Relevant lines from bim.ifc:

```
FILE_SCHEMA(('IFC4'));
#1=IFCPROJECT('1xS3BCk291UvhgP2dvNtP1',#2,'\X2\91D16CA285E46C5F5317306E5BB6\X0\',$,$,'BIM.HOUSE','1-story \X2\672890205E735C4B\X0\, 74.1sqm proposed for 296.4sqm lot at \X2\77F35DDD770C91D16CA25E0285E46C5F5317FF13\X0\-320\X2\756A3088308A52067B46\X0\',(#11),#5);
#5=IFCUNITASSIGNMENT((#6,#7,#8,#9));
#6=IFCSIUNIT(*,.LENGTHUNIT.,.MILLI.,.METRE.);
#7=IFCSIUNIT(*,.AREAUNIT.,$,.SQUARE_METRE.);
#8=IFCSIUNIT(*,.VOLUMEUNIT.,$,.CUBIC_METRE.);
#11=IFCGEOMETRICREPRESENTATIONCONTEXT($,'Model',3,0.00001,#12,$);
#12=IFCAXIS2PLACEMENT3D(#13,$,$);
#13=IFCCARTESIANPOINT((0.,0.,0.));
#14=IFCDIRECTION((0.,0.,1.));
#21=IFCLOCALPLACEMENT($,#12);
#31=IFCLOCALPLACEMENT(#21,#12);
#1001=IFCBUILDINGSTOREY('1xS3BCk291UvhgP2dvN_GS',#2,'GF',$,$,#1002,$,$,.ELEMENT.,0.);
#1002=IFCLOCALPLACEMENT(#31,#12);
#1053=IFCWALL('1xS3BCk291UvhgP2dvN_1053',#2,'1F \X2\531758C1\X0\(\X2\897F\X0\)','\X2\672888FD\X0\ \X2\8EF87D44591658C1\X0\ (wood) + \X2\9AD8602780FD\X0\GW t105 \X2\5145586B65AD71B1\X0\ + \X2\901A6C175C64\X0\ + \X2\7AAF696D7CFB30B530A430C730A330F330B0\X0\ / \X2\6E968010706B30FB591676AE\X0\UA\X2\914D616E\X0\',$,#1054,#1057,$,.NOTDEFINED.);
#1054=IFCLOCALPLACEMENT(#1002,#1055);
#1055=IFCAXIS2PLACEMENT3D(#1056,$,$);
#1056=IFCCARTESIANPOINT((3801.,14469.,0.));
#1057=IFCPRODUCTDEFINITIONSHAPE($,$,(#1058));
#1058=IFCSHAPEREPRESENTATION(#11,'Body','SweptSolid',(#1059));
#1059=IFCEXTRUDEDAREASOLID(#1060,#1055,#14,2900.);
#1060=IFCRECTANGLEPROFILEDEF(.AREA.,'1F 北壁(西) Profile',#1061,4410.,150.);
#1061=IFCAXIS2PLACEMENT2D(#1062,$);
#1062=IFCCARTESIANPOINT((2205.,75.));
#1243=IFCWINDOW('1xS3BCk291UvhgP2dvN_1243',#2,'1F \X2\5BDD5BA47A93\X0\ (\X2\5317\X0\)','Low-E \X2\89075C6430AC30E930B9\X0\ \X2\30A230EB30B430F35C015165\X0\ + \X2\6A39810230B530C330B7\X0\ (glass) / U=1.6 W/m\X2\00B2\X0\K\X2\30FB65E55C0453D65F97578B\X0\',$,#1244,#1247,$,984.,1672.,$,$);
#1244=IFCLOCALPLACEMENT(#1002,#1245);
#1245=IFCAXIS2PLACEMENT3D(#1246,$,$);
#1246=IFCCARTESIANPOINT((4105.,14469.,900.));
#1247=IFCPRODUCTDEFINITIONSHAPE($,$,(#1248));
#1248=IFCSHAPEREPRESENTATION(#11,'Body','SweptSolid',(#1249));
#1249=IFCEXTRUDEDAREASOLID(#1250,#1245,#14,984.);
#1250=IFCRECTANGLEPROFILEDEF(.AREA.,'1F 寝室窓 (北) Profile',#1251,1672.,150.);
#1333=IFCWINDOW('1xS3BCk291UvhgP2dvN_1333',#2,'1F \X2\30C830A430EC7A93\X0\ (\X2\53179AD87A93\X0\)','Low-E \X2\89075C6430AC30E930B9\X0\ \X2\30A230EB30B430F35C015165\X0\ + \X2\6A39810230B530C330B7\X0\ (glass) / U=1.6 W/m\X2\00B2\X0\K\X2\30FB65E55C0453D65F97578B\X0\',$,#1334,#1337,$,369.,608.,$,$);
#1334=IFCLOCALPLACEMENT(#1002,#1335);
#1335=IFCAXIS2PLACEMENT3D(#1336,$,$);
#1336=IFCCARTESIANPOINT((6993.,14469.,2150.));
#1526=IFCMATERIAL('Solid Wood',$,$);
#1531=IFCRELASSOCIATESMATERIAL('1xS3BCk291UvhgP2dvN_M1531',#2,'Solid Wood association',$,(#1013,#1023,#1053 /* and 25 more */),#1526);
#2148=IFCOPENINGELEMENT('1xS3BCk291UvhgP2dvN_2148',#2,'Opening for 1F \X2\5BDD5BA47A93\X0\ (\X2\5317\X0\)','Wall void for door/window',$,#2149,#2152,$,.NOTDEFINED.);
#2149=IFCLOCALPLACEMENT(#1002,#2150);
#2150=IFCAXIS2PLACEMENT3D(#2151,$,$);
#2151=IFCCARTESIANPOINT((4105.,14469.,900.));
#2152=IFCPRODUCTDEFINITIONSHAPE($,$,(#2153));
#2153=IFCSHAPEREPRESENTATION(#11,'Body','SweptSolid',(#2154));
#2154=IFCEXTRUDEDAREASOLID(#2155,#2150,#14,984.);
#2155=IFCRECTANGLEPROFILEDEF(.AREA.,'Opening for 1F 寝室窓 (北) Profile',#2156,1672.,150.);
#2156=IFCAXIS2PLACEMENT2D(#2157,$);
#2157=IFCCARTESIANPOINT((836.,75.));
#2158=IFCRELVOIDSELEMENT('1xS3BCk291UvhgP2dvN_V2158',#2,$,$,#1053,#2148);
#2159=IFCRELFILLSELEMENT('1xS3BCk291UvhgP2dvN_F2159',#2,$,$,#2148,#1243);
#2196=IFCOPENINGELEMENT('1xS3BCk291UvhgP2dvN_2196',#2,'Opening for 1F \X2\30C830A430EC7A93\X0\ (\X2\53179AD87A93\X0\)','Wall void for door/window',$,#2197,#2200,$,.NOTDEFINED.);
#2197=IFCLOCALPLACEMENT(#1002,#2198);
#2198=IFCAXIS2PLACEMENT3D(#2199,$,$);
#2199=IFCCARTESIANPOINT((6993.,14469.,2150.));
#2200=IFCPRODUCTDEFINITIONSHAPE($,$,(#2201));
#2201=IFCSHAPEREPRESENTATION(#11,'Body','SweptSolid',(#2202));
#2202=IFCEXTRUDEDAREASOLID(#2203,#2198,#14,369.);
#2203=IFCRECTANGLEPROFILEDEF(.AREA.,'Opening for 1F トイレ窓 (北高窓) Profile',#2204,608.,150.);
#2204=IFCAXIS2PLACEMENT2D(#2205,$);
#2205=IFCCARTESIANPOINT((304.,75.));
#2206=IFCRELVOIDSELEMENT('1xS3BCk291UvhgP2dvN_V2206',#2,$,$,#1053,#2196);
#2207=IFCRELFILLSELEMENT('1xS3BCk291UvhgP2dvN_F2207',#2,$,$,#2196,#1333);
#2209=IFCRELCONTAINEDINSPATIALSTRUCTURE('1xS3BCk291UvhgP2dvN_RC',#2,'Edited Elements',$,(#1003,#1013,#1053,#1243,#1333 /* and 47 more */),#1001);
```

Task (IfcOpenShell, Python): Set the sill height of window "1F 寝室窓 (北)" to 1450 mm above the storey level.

```python
import numpy as np
import ifcopenshell
import ifcopenshell.api.geometry
import ifcopenshell.geom
import ifcopenshell.util.element
import ifcopenshell.util.placement
import ifcopenshell.util.shape
import ifcopenshell.util.unit

model = ifcopenshell.open("bim.ifc")
unit_scale = ifcopenshell.util.unit.calculate_unit_scale(model)

window = model.by_id(1243)
opening = window.FillsVoids[0].RelatingOpeningElement
storey = ifcopenshell.util.element.get_container(window, ifc_class="IfcBuildingStorey")
level = ifcopenshell.util.placement.get_local_placement(storey.ObjectPlacement)[2, 3]

# The opening's origin need not be at the sill, so measure its lowest point.
shape = ifcopenshell.geom.create_shape(ifcopenshell.geom.settings(), opening)
bottom = ifcopenshell.util.shape.get_shape_bottom_elevation(shape, shape.geometry) / unit_scale
dz = level + 1450.0 - bottom

shift = np.array([0.0, 0.0, dz])
# The window is not placed relative to its opening, so move both.
for product in (opening, window):
    matrix = ifcopenshell.util.placement.get_local_placement(product.ObjectPlacement)
    matrix[:3, 3] += shift
    ifcopenshell.api.geometry.edit_object_placement(model, product=product, matrix=matrix, is_si=False)

print(f"moved by {dz * unit_scale:+.3f} m")

model.write("bim_updated.ifc")
```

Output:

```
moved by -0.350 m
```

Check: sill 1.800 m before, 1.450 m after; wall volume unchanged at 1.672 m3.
